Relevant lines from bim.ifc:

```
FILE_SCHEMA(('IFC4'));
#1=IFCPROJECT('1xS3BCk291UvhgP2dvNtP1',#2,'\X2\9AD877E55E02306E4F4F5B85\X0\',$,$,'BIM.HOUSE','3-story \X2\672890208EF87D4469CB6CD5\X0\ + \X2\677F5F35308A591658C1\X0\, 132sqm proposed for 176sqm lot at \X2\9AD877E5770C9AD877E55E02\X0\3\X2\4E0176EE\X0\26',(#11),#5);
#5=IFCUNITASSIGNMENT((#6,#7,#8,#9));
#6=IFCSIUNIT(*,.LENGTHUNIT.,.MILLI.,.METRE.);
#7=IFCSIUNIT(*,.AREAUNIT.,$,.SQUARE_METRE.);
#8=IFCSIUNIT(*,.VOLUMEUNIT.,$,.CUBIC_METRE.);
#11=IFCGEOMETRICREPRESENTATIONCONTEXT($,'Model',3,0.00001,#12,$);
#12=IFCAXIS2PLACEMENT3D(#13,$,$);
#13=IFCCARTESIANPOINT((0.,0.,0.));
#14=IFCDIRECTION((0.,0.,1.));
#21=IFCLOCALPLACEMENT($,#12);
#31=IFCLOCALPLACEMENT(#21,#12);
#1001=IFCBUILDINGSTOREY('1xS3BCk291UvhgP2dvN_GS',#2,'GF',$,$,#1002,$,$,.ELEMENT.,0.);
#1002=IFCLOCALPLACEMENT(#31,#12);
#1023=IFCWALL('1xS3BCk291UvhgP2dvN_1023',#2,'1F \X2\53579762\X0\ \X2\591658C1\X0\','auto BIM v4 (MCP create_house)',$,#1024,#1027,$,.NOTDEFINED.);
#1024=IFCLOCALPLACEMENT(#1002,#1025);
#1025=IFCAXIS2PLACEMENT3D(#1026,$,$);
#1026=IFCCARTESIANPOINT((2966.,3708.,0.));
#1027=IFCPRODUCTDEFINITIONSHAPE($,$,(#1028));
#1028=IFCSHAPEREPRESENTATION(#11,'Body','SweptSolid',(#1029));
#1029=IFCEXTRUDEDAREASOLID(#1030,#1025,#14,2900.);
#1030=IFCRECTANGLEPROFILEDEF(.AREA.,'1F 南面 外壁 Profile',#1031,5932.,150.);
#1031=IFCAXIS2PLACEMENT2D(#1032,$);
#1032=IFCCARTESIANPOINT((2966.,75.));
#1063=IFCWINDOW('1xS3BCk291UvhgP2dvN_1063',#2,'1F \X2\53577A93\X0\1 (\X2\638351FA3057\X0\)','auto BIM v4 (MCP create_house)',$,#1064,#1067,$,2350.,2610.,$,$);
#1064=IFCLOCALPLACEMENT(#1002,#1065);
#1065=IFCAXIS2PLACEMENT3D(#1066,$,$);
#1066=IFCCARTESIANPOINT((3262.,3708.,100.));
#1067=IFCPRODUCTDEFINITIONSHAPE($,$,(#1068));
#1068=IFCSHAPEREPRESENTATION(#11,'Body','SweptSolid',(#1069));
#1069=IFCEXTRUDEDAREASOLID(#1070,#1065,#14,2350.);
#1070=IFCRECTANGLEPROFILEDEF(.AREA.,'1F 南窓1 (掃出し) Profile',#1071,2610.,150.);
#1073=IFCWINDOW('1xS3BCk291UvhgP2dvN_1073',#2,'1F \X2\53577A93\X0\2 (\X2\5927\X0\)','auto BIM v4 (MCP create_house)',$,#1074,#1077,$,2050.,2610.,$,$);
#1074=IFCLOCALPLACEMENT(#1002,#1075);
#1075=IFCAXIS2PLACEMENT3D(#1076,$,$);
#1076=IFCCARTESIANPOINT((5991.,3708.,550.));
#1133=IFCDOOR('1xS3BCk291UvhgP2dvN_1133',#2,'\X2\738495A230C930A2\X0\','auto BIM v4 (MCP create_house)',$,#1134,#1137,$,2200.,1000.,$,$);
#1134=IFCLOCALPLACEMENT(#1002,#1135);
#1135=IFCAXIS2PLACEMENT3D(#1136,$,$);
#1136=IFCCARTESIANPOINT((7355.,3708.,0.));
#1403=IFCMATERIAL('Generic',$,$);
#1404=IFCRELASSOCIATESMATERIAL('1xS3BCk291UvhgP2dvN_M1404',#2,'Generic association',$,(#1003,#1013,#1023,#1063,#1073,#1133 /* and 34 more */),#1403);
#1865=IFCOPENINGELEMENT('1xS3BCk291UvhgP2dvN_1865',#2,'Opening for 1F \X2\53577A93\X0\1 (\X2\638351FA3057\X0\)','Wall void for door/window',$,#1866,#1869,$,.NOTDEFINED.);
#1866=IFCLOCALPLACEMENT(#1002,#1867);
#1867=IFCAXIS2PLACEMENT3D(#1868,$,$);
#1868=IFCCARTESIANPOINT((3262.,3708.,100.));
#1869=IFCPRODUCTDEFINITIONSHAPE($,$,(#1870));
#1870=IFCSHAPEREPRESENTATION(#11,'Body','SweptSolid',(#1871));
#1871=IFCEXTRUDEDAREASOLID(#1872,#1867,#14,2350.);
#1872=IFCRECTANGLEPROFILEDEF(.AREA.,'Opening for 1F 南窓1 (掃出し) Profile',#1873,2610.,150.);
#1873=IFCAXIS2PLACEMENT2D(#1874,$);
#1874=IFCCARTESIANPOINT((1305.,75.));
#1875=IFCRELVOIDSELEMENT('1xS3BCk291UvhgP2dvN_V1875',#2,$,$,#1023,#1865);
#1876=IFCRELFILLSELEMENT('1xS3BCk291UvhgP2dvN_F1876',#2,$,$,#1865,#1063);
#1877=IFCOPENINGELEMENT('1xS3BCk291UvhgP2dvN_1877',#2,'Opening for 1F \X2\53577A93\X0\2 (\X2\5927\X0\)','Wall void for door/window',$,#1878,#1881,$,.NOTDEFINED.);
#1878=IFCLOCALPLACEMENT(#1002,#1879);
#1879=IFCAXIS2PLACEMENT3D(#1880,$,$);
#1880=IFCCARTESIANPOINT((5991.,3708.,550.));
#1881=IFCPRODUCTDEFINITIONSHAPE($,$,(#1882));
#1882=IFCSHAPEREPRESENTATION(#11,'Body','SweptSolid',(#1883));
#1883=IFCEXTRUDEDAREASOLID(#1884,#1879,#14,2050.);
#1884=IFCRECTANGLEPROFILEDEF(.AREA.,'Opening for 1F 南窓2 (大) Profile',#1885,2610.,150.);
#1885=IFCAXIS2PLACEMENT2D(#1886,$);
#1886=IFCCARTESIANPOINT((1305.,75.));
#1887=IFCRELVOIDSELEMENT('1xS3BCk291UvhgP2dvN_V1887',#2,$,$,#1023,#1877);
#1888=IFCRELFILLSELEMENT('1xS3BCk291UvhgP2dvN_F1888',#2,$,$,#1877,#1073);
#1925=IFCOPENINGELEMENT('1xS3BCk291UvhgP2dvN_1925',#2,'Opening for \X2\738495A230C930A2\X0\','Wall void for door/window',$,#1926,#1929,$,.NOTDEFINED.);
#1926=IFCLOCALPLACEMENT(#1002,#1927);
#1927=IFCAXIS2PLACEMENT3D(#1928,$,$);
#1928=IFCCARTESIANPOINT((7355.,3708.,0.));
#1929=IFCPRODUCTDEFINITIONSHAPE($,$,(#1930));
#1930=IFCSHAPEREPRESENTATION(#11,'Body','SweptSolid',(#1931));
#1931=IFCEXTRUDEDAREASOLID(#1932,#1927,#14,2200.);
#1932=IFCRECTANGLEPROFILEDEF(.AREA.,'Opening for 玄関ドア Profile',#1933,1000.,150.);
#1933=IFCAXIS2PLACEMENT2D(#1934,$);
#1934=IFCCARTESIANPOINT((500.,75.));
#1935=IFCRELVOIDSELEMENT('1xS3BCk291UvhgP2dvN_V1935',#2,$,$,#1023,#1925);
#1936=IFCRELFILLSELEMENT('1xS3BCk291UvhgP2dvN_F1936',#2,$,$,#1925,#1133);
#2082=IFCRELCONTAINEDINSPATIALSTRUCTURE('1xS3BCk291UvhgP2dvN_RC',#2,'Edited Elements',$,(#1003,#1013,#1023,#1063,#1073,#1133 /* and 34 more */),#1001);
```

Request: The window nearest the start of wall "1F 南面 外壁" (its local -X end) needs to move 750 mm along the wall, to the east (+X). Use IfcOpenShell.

```python
import ifcopenshell
import ifcopenshell.api.geometry
import ifcopenshell.util.placement

model = ifcopenshell.open("bim.ifc")

window = model.by_id(1063)
opening = window.FillsVoids[0].RelatingOpeningElement
wall = opening.VoidsElements[0].RelatingBuildingElement

wall_matrix = ifcopenshell.util.placement.get_local_placement(wall.ObjectPlacement)
shift = wall_matrix[:3, 0] * 750.0
before = ifcopenshell.util.placement.get_local_placement(window.ObjectPlacement)[:3, 3].copy()

# The window is not placed relative to its opening, so move both.
for product in (opening, window):
    matrix = ifcopenshell.util.placement.get_local_placement(product.ObjectPlacement)
    matrix[:3, 3] += shift
    ifcopenshell.api.geometry.edit_object_placement(model, product=product, matrix=matrix, is_si=False)

after = ifcopenshell.util.placement.get_local_placement(window.ObjectPlacement)[:3, 3]
print("window moved by", (after - before).round(3) + 0.0)

model.write("bim_rev.ifc")
```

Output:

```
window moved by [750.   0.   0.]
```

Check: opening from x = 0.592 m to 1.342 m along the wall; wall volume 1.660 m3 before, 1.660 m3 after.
